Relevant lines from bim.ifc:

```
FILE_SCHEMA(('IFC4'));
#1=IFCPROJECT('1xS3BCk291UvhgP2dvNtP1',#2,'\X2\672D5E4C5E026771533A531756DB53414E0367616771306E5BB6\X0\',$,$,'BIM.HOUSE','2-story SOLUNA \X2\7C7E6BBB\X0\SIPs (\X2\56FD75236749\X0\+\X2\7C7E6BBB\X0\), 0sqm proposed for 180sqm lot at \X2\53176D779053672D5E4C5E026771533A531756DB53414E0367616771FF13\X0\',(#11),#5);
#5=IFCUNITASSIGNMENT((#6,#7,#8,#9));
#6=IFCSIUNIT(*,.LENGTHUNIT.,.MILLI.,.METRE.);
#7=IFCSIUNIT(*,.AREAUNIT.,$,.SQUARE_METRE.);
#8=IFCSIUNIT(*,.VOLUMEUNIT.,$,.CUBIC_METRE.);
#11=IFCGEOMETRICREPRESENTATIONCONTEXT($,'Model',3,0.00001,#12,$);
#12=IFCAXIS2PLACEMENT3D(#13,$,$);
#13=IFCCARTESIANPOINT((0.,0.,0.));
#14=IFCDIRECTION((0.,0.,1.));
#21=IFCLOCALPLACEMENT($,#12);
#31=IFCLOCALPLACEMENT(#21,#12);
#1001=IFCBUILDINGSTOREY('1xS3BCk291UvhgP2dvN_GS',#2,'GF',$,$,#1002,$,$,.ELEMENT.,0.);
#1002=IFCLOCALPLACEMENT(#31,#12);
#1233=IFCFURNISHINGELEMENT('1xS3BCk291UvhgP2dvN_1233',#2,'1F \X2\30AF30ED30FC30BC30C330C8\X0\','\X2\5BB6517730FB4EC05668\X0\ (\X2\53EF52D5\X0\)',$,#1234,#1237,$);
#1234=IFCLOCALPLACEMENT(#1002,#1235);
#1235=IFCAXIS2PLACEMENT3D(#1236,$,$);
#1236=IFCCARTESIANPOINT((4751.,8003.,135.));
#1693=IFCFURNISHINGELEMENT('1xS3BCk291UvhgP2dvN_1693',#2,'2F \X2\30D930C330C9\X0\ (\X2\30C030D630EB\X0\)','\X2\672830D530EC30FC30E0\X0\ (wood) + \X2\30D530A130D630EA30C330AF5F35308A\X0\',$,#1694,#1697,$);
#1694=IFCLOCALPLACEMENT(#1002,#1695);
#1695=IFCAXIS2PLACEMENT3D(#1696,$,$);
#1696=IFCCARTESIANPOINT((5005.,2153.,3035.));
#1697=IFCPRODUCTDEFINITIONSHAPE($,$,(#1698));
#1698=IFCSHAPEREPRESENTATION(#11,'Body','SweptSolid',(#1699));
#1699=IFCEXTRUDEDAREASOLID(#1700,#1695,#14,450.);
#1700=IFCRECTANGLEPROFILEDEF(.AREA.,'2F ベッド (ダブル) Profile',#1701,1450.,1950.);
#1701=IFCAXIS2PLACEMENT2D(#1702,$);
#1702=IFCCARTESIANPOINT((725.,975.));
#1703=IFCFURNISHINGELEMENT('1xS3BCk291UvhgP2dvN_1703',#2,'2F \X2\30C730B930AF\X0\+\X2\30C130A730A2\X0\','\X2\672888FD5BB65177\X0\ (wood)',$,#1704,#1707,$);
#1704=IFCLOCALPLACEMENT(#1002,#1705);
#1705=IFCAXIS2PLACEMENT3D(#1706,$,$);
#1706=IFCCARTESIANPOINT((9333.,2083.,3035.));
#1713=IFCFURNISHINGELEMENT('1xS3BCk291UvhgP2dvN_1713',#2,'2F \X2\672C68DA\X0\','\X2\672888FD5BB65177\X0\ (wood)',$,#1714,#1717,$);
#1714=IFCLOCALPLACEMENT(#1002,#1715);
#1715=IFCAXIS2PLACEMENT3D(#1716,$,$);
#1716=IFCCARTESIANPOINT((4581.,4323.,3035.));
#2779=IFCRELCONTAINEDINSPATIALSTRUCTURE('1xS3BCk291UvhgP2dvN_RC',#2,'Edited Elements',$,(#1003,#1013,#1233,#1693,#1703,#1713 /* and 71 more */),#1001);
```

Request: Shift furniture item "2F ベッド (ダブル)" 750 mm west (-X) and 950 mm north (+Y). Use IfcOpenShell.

```python
import ifcopenshell
import ifcopenshell.api.geometry
import ifcopenshell.util.placement
import ifcopenshell.util.unit

model = ifcopenshell.open("bim.ifc")
unit_scale = ifcopenshell.util.unit.calculate_unit_scale(model)

item = model.by_id(1693)
matrix = ifcopenshell.util.placement.get_local_placement(item.ObjectPlacement)
matrix[0, 3] -= 0.75 / unit_scale
matrix[1, 3] += 0.95 / unit_scale
ifcopenshell.api.geometry.edit_object_placement(model, product=item, matrix=matrix, is_si=False)

print(ifcopenshell.util.placement.get_local_placement(item.ObjectPlacement).round(3) + 0.0)

model.write("bim_updated.ifc")
```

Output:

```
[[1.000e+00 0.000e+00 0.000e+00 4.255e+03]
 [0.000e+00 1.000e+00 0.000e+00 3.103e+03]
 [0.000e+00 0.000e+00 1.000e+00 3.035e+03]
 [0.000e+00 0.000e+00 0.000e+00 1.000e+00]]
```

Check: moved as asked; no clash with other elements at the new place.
